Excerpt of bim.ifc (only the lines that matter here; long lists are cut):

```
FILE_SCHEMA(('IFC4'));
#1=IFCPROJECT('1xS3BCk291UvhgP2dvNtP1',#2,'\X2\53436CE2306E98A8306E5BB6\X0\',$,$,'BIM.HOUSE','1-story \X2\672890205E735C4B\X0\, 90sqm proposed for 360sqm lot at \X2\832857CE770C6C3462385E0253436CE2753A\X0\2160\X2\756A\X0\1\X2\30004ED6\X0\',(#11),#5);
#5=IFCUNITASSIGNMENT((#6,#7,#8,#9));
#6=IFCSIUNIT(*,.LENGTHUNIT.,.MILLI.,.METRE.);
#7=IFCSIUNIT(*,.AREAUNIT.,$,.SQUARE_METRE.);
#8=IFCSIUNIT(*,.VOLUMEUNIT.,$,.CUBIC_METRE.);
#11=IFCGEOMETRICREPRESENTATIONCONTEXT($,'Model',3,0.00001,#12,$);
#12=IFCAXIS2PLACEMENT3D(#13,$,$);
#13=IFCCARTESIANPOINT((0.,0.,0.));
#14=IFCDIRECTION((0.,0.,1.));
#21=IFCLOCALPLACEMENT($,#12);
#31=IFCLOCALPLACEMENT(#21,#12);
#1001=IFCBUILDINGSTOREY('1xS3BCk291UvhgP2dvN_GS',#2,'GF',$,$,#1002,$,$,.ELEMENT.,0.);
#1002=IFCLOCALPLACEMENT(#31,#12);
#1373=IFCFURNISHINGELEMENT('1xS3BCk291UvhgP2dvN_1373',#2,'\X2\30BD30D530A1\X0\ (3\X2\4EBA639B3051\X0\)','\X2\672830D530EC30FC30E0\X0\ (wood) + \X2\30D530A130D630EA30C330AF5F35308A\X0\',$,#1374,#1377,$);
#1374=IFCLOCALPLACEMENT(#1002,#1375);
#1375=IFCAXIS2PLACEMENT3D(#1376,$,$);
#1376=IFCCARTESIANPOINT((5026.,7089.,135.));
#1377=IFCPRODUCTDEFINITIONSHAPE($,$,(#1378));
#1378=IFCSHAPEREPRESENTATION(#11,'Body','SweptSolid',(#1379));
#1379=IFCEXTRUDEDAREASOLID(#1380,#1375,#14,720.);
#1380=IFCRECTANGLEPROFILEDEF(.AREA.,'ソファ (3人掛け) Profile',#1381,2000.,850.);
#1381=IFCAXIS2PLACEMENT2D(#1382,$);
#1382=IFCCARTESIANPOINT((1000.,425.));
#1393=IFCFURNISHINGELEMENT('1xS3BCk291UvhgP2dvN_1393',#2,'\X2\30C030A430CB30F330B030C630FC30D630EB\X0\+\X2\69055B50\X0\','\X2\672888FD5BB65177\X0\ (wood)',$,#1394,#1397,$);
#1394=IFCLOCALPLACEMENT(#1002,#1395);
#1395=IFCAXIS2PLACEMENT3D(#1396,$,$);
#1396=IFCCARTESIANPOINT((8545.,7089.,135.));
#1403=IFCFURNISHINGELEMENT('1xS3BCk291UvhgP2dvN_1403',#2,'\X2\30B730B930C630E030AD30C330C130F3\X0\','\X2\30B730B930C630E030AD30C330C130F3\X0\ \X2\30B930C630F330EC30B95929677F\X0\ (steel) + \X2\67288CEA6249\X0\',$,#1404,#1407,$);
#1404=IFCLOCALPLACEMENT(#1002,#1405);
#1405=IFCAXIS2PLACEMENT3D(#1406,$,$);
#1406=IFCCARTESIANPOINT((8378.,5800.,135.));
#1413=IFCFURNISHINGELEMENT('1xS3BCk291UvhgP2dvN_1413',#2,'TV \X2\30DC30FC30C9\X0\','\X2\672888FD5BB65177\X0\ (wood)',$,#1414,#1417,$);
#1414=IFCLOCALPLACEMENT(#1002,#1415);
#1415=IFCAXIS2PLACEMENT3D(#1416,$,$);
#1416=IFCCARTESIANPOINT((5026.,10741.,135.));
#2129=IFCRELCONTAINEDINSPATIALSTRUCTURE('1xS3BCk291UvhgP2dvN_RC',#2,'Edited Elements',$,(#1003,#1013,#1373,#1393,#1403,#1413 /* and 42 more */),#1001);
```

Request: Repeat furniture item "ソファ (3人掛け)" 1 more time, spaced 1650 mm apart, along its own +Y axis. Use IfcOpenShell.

```python
import ifcopenshell
import ifcopenshell.api.geometry
import ifcopenshell.api.root
import ifcopenshell.util.element
import ifcopenshell.util.placement
import ifcopenshell.util.unit

model = ifcopenshell.open("bim.ifc")
unit_scale = ifcopenshell.util.unit.calculate_unit_scale(model)


def reuse_history(source, copy):
    """copy_class also copies each property set's owner history, people and application; keep the originals."""
    for rel in copy.IsDefinedBy:
        if rel.is_a("IfcRelDefinesByProperties") and (history := rel.RelatingPropertyDefinition.OwnerHistory):
            rel.RelatingPropertyDefinition.OwnerHistory = source.OwnerHistory
            ifcopenshell.util.element.remove_deep2(model, history)


source = model.by_id(1373)
base = ifcopenshell.util.placement.get_local_placement(source.ObjectPlacement)
step = base[:3, 1] * 1.65 / unit_scale

for i in range(1, 2):
    copy = ifcopenshell.api.root.copy_class(model, product=source)
    copy.Representation = ifcopenshell.util.element.copy_deep(
        model, source.Representation, exclude=["IfcGeometricRepresentationContext", "IfcRepresentationMap"]
    )
    reuse_history(source, copy)
    matrix = base.copy()
    matrix[:3, 3] += i * step
    print("added at", matrix[:3, 3].round(3) + 0.0)
    ifcopenshell.api.geometry.edit_object_placement(model, product=copy, matrix=matrix, is_si=False)

model.write("bim_rev.ifc")
```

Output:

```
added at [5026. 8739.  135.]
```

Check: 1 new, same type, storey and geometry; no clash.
